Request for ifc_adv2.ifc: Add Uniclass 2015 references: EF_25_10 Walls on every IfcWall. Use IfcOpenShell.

First a look at what the model holds.

```python
import ifcopenshell

model = ifcopenshell.open("ifc_adv2.ifc")
print(model.schema)
print("classifications:", [c.Name for c in model.by_type("IfcClassification")])
for ifc_class in ("IfcDoor", "IfcRoof", "IfcStair", "IfcWall", "IfcWindow"):
    print(ifc_class, len(model.by_type(ifc_class)))
```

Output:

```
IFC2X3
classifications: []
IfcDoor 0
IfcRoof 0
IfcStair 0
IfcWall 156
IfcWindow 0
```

```python
import ifcopenshell
import ifcopenshell.api.classification

model = ifcopenshell.open("ifc_adv2.ifc")

# IFC2X3 requires Source and Edition and has no link from the project to the system.
system = model.create_entity("IfcClassification", Source="NBS", Edition="2015", Name="Uniclass 2015")

codes = {
    "IfcWall": ("EF_25_10", "Walls"),
}
for ifc_class, (code, name) in codes.items():
    products = model.by_type(ifc_class)
    ifcopenshell.api.classification.add_reference(
        model, products=products, classification=system, identification=code, name=name
    )
    print(code, len(products))

model.write("ifc_adv2_edited.ifc")
```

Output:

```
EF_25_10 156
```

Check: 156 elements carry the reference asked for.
